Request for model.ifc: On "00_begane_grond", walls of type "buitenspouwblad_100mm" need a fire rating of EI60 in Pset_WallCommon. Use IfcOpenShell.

First a look at what the model holds.

```python
import ifcopenshell
import ifcopenshell.util.element

model = ifcopenshell.open("model.ifc")
print(model.schema)
storey = next(s for s in model.by_type("IfcBuildingStorey") if s.Name == "00_begane_grond")
walls = [e for e in ifcopenshell.util.element.get_decomposition(storey) if e.is_a("IfcWall")]
seen = {}
for e in walls:
    element_type = ifcopenshell.util.element.get_type(e)
    key = (element_type.Name if element_type != e and element_type else None, ifcopenshell.util.element.get_pset(e, "Pset_WallCommon", "FireRating"))
    seen[key] = seen.get(key, 0) + 1
for (name, value), count in sorted(seen.items(), key=str):
    print(count, "x", name, "|", value)
```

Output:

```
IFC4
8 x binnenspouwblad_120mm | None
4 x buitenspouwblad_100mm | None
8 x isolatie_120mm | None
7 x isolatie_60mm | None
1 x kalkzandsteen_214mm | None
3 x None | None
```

```python
import ifcopenshell
import ifcopenshell.api.pset
import ifcopenshell.util.element

model = ifcopenshell.open("model.ifc")

storey = next(s for s in model.by_type("IfcBuildingStorey") if s.Name == "00_begane_grond")
walls = [e for e in ifcopenshell.util.element.get_decomposition(storey) if e.is_a("IfcWall")]

count = 0
for e in walls:
    element_type = ifcopenshell.util.element.get_type(e)
    if element_type in (None, e) or element_type.Name != "buitenspouwblad_100mm":
        continue
    # add_pset returns the element's existing set when there is one.
    pset = ifcopenshell.api.pset.add_pset(model, product=e, name="Pset_WallCommon")
    ifcopenshell.api.pset.edit_pset(model, pset=pset, properties={"FireRating": "EI60"})
    count += 1

print(count, "walls updated")

model.write("model_rev.ifc")
```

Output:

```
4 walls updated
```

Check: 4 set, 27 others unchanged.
